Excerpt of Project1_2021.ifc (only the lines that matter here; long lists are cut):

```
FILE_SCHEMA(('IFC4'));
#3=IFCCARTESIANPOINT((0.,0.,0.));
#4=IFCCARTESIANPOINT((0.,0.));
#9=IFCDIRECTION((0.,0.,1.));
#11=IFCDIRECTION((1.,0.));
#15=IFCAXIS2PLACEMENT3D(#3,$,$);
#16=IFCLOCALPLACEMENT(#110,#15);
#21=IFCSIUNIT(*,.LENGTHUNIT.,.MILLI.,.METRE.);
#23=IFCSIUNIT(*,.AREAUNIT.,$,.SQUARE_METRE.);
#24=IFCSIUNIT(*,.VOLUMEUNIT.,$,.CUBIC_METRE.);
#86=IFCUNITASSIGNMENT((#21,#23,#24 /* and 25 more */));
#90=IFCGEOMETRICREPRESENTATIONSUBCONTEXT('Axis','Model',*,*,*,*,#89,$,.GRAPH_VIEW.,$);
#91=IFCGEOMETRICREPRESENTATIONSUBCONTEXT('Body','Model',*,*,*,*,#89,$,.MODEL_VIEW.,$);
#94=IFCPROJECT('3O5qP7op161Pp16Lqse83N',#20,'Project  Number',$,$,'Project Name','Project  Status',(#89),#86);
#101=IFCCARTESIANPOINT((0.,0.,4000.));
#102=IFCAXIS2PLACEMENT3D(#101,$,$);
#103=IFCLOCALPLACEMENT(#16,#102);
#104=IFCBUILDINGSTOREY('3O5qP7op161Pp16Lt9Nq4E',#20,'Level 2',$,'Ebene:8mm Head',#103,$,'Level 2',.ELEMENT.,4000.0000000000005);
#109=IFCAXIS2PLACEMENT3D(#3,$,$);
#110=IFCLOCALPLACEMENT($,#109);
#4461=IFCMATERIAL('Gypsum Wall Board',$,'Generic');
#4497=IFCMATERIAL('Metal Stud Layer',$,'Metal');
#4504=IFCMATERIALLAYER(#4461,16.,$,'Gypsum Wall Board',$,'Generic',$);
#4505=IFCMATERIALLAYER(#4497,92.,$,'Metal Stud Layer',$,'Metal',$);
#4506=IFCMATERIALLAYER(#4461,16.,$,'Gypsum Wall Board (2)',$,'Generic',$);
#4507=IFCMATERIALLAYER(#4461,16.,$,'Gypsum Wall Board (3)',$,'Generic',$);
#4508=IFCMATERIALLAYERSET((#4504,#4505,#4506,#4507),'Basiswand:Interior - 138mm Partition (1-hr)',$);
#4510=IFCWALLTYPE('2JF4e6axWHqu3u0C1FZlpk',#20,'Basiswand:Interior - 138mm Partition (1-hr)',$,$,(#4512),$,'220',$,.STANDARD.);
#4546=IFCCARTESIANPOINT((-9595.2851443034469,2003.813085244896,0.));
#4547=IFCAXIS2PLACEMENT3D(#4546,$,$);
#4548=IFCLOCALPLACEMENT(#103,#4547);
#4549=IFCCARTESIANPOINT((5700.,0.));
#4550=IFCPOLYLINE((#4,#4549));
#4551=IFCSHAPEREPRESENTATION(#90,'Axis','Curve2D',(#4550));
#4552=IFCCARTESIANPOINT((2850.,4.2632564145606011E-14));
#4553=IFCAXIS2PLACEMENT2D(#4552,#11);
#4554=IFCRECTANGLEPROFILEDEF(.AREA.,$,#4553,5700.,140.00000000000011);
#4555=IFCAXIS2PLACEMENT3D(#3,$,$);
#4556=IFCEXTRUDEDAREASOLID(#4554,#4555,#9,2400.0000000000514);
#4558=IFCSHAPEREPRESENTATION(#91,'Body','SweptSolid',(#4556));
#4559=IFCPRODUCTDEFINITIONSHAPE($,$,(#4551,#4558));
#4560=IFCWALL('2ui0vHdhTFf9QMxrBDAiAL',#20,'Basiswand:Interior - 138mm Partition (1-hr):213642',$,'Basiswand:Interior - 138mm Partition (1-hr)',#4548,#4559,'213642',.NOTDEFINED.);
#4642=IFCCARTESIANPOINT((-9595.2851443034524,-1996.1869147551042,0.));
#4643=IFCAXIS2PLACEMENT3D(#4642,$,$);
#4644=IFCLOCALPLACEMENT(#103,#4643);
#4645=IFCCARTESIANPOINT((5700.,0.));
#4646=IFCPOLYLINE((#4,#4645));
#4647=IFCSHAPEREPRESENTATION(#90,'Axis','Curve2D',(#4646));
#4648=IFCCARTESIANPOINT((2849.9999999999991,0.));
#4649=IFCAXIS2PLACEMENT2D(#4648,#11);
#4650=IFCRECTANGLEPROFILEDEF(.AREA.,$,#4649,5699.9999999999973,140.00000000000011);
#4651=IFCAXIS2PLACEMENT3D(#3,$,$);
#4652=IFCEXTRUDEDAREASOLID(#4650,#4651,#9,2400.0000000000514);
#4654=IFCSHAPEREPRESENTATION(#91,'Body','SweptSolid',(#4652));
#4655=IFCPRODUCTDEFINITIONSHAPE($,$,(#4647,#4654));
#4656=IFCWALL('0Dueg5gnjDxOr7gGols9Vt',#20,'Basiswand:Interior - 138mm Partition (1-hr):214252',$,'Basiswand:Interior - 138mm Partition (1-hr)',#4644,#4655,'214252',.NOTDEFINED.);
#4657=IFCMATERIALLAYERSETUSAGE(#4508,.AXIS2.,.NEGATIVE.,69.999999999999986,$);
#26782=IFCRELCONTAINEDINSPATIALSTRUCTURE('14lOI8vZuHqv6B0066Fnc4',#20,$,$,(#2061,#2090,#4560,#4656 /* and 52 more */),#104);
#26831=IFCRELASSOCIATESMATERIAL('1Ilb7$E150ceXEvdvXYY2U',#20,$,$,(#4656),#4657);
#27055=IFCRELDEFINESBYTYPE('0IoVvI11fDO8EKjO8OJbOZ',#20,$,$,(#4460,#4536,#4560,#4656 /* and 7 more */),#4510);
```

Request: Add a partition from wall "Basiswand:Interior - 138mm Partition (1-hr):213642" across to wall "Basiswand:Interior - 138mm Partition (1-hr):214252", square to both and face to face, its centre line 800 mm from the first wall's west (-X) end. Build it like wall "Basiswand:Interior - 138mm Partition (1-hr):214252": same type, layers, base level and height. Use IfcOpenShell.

```python
import numpy as np
import ifcopenshell
import ifcopenshell.api.geometry
import ifcopenshell.api.material
import ifcopenshell.api.pset
import ifcopenshell.api.root
import ifcopenshell.api.spatial
import ifcopenshell.api.type
import ifcopenshell.geom
import ifcopenshell.util.element
import ifcopenshell.util.placement
import ifcopenshell.util.representation
import ifcopenshell.util.shape
import ifcopenshell.util.unit

model = ifcopenshell.open("Project1_2021.ifc")
unit_scale = ifcopenshell.util.unit.calculate_unit_scale(model)
settings = ifcopenshell.geom.settings()
settings.set("use-world-coords", True)

start_wall = model.by_id(4560)
end_wall = model.by_guid("0Dueg5gnjDxOr7gGols9Vt")
like = model.by_guid("0Dueg5gnjDxOr7gGols9Vt")
matrix = ifcopenshell.util.placement.get_local_placement(start_wall.ObjectPlacement)
matrix[:3, 3] *= unit_scale


def extent(element):
    """Bounding box in the first wall's axes, in metres."""
    shape = ifcopenshell.geom.create_shape(settings, element)
    points = (ifcopenshell.util.shape.get_vertices(shape.geometry) - matrix[:3, 3]) @ matrix[:3, :3]
    return points.min(axis=0), points.max(axis=0)


y_start = extent(start_wall)[0][1]
y_end = extent(end_wall)[1][1]
like_min, like_max = extent(like)
length, height = float(abs(y_end - y_start)), float(like_max[2] - like_min[2])
layer_set = ifcopenshell.util.element.get_material(like, should_skip_usage=True)
thickness = sum(layer.LayerThickness for layer in layer_set.MaterialLayers) * unit_scale

wall = ifcopenshell.api.root.create_entity(model, ifc_class="IfcWall", name="New partition")
storey = ifcopenshell.util.element.get_container(like)
ifcopenshell.api.spatial.assign_container(model, products=[wall], relating_structure=storey)
ifcopenshell.api.type.assign_type(
    model, related_objects=[wall], relating_type=ifcopenshell.util.element.get_type(like), should_map_representations=False
)
rel = ifcopenshell.api.material.assign_material(
    model, products=[wall], type="IfcMaterialLayerSetUsage", material=layer_set
)
rel.RelatingMaterial.OffsetFromReferenceLine = -thickness / 2 / unit_scale
pset = ifcopenshell.api.pset.add_pset(model, product=wall, name="Pset_WallCommon")
ifcopenshell.api.pset.edit_pset(model, pset=pset, properties={"IsExternal": False, "LoadBearing": False})

# The axis runs down the middle of the wall.
axis = ifcopenshell.api.geometry.add_axis_representation(
    model, context=ifcopenshell.util.representation.get_context(model, "Model", "Axis"), axis=[(0.0, 0.0), (length, 0.0)]
)
body = ifcopenshell.api.geometry.add_wall_representation(
    model,
    context=ifcopenshell.util.representation.get_context(model, "Model", "Body", "MODEL_VIEW"),
    length=length,
    height=height,
    thickness=thickness,
    offset=-thickness / 2,
)
for representation in (axis, body):
    ifcopenshell.api.geometry.assign_representation(model, product=wall, representation=representation)

placement = matrix @ ifcopenshell.util.placement.rotation(-90, "Z")
placement[:, 3] = matrix @ np.array([extent(start_wall)[0][0] + 0.8, y_start, like_min[2], 1.0])
ifcopenshell.api.geometry.edit_object_placement(model, product=wall, matrix=placement)

print(f"partition {length:.3f} m long, {height:.3f} m high, {thickness:.3f} m thick")

model.write("Project1_2021_rev.ifc")
```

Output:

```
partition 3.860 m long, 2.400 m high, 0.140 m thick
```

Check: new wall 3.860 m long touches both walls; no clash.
